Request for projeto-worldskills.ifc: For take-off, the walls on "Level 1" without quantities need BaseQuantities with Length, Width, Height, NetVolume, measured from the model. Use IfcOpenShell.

First a look at what the model holds.

```python
import ifcopenshell
import ifcopenshell.util.element
import ifcopenshell.util.unit

model = ifcopenshell.open("projeto-worldskills.ifc")
print(model.schema)
for unit_type in ("LENGTHUNIT", "AREAUNIT", "VOLUMEUNIT"):
    print(unit_type, ifcopenshell.util.unit.calculate_unit_scale(model, unit_type))
storey = next(s for s in model.by_type("IfcBuildingStorey") if s.Name == "Level 1")
walls = [e for e in ifcopenshell.util.element.get_decomposition(storey) if e.is_a("IfcWall")]
for e in sorted(walls, key=lambda e: e.id()):
    print(e.id(), e.is_a(), e.Name, list(ifcopenshell.util.element.get_psets(e, qtos_only=True)), sep=" | ")
```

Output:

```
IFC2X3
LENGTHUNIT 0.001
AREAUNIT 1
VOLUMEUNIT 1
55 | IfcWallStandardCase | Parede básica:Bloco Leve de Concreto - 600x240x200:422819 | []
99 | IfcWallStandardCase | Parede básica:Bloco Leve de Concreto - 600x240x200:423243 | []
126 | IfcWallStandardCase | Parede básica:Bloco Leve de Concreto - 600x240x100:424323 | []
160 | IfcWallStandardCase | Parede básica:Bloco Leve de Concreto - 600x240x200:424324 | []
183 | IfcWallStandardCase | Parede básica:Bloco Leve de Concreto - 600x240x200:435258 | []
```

```python
import ifcopenshell
import ifcopenshell.api.pset
import ifcopenshell.geom
import ifcopenshell.util.element
import ifcopenshell.util.shape
import ifcopenshell.util.unit

model = ifcopenshell.open("projeto-worldskills.ifc")
unit_scale = ifcopenshell.util.unit.calculate_unit_scale(model)
volume_scale = ifcopenshell.util.unit.calculate_unit_scale(model, "VOLUMEUNIT")
settings = ifcopenshell.geom.settings()

storey = next(s for s in model.by_type("IfcBuildingStorey") if s.Name == "Level 1")
walls = [e for e in ifcopenshell.util.element.get_decomposition(storey) if e.is_a("IfcWall")]

for e in sorted(walls, key=lambda e: e.id()):
    if ifcopenshell.util.element.get_psets(e, qtos_only=True, should_inherit=False):
        continue
    # Geometry comes back in metres, in the element's own axes.
    shape = ifcopenshell.geom.create_shape(settings, e)
    values = {
        "Length": ifcopenshell.util.shape.get_x(shape.geometry) / unit_scale,
        "Width": ifcopenshell.util.shape.get_y(shape.geometry) / unit_scale,
        "Height": ifcopenshell.util.shape.get_z(shape.geometry) / unit_scale,
        "NetVolume": ifcopenshell.util.shape.get_volume(shape.geometry) / volume_scale,
    }
    qto = ifcopenshell.api.pset.add_qto(model, product=e, name="BaseQuantities")
    ifcopenshell.api.pset.edit_qto(model, qto=qto, properties=values)
    print(e.id(), {k: round(v, 3) for k, v in values.items()})

model.write("projeto-worldskills_updated.ifc")
```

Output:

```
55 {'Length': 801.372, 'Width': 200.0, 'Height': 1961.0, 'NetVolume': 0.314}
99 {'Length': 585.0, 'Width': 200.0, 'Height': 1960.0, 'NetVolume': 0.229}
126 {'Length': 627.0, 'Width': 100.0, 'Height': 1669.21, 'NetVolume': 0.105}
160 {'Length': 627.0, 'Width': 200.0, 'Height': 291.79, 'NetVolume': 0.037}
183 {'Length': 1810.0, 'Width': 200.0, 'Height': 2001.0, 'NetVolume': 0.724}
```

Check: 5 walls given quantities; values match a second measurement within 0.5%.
